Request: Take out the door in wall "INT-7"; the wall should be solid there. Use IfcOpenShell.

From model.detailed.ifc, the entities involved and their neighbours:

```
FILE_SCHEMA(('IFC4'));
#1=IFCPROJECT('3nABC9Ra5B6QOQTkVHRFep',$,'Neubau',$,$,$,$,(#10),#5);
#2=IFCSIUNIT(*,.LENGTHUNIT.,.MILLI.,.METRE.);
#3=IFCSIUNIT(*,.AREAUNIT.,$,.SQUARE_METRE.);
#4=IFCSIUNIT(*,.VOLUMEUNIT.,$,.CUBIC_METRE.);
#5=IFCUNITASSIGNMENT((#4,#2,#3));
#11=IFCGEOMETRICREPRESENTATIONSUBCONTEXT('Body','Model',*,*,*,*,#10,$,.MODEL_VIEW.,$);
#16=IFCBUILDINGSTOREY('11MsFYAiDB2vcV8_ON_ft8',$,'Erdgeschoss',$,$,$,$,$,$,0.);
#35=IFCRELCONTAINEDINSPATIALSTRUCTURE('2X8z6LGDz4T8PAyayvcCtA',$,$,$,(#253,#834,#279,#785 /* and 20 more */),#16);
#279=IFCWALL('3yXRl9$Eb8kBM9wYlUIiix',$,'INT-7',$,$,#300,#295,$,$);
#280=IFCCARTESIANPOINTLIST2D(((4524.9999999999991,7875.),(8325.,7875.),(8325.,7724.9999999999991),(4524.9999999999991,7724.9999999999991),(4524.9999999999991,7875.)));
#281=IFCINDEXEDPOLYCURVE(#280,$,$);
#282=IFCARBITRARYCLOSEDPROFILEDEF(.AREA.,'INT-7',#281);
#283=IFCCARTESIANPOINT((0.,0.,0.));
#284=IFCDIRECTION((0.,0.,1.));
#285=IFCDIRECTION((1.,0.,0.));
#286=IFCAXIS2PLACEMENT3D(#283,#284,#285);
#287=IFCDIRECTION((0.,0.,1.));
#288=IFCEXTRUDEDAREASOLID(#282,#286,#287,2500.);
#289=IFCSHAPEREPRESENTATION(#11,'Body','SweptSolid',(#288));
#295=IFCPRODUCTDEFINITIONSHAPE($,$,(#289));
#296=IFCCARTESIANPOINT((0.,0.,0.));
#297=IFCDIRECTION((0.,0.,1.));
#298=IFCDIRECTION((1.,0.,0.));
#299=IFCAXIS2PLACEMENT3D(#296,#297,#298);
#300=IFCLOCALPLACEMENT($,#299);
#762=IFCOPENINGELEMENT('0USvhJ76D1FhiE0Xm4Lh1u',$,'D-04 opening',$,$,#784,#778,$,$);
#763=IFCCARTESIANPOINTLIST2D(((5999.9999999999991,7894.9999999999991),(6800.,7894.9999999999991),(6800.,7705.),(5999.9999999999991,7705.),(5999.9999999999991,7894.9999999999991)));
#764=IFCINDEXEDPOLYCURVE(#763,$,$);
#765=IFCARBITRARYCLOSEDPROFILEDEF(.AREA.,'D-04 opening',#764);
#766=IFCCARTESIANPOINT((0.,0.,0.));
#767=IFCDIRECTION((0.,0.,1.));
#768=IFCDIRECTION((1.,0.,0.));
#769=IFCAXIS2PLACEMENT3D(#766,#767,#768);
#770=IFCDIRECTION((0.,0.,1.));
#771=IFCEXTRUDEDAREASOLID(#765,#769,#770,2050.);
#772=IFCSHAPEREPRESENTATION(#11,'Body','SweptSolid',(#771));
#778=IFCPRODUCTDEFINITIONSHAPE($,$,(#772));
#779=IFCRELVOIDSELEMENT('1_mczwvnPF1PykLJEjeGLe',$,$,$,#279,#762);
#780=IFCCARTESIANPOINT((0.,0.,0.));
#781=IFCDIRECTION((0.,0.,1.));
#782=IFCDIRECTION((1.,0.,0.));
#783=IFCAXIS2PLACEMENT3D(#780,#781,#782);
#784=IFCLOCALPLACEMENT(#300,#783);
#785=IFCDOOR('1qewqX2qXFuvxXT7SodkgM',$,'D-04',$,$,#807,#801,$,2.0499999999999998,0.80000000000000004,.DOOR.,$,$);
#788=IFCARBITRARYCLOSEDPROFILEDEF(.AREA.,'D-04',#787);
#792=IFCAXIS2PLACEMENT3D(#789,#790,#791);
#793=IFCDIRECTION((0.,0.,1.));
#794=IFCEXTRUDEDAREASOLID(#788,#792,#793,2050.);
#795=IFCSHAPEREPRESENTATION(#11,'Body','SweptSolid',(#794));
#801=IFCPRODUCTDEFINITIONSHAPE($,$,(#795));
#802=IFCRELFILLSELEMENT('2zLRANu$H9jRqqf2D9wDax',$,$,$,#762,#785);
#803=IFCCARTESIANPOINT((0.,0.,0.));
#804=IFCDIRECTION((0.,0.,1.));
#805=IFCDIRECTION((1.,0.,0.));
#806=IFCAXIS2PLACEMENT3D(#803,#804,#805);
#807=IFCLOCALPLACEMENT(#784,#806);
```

```python
import ifcopenshell
import ifcopenshell.api.feature
import ifcopenshell.api.root
import ifcopenshell.geom
import ifcopenshell.util.shape

model = ifcopenshell.open("model.detailed.ifc")
settings = ifcopenshell.geom.settings()


def volume(element):
    """Net volume in cubic metres, openings subtracted."""
    shape = ifcopenshell.geom.create_shape(settings, element)
    return ifcopenshell.util.shape.get_volume(shape.geometry)


door = model.by_guid("1qewqX2qXFuvxXT7SodkgM")
opening = door.FillsVoids[0].RelatingOpeningElement
wall = opening.VoidsElements[0].RelatingBuildingElement
before = volume(wall)

ifcopenshell.api.root.remove_product(model, product=door)
ifcopenshell.api.feature.remove_feature(model, feature=opening)

after = volume(wall)

print(f"wall volume {before:.3f} -> {after:.3f} m3")

model.write("model.detailed_rev.ifc")
```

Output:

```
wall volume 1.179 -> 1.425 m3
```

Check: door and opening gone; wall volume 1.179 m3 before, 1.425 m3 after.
